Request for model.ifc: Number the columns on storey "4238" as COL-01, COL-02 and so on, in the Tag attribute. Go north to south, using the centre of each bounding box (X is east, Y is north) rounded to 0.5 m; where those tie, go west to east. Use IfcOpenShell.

First a look at what the model holds.

```python
import ifcopenshell
import ifcopenshell.util.element
import ifcopenshell.util.placement

model = ifcopenshell.open("model.ifc")
print(model.schema)
storey = next(s for s in model.by_type("IfcBuildingStorey") if s.Name == "4238")
columns = [e for e in ifcopenshell.util.element.get_decomposition(storey) if e.is_a("IfcColumn")]
for e in sorted(columns, key=lambda e: e.id()):
    origin = ifcopenshell.util.placement.get_local_placement(e.ObjectPlacement)[:3, 3]
    print(e.id(), e.Tag, e.Name, origin.round(2) + 0.0, sep=" | ")
```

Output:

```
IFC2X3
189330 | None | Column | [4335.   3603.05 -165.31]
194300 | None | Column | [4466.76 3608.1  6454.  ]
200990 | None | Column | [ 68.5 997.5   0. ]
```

```python
import ifcopenshell
import ifcopenshell.geom
import ifcopenshell.util.element
import ifcopenshell.util.shape

model = ifcopenshell.open("model.ifc")
settings = ifcopenshell.geom.settings()
settings.set("use-world-coords", True)


def centre(element):
    shape = ifcopenshell.geom.create_shape(settings, element)
    return ifcopenshell.util.shape.get_bbox_centroid(shape.geometry)


storey = next(s for s in model.by_type("IfcBuildingStorey") if s.Name == "4238")
columns = [e for e in ifcopenshell.util.element.get_decomposition(storey) if e.is_a("IfcColumn")]

# Insertion points can sit at a corner or the storey origin, so sort by the geometry (in metres).
centres = {e: centre(e) for e in columns}
columns.sort(key=lambda e: (-round(centres[e][1] / 0.5), centres[e][0]))

for i, e in enumerate(columns, start=1):
    number = f"COL-{i:02d}"
    e.Tag = number
    print(e.id(), number)

model.write("model_edited.ifc")
```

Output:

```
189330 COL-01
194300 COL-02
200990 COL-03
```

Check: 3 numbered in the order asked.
